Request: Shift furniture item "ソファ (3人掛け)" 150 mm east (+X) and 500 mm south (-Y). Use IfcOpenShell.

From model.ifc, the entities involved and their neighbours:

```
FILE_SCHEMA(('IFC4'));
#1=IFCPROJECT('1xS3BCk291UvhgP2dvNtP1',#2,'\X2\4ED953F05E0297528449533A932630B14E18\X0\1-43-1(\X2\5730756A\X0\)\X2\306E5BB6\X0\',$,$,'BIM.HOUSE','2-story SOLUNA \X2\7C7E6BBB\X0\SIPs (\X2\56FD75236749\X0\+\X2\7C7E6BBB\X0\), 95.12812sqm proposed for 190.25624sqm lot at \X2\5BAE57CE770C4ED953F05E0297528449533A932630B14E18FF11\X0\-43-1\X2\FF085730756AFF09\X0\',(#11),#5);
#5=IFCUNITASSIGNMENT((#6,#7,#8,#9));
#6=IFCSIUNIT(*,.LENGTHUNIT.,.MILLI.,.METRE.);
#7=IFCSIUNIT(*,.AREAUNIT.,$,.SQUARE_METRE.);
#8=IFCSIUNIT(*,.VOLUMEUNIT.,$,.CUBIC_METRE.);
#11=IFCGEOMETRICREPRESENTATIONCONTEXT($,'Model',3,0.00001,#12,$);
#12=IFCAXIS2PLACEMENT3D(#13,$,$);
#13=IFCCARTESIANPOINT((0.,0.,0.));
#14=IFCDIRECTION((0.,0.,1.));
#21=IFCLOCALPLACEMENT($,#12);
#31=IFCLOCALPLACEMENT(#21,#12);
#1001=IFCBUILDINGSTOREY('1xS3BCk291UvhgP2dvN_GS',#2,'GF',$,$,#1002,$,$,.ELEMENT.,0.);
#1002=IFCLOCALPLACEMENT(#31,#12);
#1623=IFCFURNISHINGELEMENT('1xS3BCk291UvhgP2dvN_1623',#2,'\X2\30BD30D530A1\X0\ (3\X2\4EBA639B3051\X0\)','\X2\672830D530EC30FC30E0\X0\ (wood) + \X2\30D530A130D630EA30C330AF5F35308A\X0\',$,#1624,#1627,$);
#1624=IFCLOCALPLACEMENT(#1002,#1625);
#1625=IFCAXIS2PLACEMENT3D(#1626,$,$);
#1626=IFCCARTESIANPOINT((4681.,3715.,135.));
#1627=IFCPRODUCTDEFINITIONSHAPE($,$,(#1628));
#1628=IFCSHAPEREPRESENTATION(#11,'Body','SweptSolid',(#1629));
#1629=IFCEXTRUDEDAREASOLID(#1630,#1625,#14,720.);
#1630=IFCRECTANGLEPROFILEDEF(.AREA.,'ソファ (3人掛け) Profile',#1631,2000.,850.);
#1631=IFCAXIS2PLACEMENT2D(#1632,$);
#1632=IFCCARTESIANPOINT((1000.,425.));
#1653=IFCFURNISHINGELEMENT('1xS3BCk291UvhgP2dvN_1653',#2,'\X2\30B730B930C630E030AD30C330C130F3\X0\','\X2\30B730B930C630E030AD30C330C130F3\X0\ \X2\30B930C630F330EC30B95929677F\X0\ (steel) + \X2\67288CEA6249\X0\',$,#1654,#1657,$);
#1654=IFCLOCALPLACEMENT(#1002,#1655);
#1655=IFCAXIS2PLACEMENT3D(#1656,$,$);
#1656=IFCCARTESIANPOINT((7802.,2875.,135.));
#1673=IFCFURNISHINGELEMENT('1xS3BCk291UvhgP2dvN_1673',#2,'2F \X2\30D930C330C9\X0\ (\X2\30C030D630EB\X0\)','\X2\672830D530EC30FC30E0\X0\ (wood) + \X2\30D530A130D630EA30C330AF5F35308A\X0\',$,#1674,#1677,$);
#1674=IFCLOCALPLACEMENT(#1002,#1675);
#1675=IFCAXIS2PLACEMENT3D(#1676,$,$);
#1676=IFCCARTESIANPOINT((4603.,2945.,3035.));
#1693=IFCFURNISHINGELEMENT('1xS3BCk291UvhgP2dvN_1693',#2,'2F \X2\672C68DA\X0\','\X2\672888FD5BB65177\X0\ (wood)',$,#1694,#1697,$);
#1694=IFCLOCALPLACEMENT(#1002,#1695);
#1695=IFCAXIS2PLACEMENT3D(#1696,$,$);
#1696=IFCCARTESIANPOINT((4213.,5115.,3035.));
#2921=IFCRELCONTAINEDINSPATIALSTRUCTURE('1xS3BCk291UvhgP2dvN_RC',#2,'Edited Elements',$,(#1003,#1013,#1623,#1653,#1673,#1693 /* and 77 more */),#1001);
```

```python
import ifcopenshell
import ifcopenshell.api.geometry
import ifcopenshell.util.placement
import ifcopenshell.util.unit

model = ifcopenshell.open("model.ifc")
unit_scale = ifcopenshell.util.unit.calculate_unit_scale(model)

item = model.by_id(1623)
matrix = ifcopenshell.util.placement.get_local_placement(item.ObjectPlacement)
matrix[0, 3] += 0.15 / unit_scale
matrix[1, 3] -= 0.5 / unit_scale
ifcopenshell.api.geometry.edit_object_placement(model, product=item, matrix=matrix, is_si=False)

print(ifcopenshell.util.placement.get_local_placement(item.ObjectPlacement).round(3) + 0.0)

model.write("model-out.ifc")
```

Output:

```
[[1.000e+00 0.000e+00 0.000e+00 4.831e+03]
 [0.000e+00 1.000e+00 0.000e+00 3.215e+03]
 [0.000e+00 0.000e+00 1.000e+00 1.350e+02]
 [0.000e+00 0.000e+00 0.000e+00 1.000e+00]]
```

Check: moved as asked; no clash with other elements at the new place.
